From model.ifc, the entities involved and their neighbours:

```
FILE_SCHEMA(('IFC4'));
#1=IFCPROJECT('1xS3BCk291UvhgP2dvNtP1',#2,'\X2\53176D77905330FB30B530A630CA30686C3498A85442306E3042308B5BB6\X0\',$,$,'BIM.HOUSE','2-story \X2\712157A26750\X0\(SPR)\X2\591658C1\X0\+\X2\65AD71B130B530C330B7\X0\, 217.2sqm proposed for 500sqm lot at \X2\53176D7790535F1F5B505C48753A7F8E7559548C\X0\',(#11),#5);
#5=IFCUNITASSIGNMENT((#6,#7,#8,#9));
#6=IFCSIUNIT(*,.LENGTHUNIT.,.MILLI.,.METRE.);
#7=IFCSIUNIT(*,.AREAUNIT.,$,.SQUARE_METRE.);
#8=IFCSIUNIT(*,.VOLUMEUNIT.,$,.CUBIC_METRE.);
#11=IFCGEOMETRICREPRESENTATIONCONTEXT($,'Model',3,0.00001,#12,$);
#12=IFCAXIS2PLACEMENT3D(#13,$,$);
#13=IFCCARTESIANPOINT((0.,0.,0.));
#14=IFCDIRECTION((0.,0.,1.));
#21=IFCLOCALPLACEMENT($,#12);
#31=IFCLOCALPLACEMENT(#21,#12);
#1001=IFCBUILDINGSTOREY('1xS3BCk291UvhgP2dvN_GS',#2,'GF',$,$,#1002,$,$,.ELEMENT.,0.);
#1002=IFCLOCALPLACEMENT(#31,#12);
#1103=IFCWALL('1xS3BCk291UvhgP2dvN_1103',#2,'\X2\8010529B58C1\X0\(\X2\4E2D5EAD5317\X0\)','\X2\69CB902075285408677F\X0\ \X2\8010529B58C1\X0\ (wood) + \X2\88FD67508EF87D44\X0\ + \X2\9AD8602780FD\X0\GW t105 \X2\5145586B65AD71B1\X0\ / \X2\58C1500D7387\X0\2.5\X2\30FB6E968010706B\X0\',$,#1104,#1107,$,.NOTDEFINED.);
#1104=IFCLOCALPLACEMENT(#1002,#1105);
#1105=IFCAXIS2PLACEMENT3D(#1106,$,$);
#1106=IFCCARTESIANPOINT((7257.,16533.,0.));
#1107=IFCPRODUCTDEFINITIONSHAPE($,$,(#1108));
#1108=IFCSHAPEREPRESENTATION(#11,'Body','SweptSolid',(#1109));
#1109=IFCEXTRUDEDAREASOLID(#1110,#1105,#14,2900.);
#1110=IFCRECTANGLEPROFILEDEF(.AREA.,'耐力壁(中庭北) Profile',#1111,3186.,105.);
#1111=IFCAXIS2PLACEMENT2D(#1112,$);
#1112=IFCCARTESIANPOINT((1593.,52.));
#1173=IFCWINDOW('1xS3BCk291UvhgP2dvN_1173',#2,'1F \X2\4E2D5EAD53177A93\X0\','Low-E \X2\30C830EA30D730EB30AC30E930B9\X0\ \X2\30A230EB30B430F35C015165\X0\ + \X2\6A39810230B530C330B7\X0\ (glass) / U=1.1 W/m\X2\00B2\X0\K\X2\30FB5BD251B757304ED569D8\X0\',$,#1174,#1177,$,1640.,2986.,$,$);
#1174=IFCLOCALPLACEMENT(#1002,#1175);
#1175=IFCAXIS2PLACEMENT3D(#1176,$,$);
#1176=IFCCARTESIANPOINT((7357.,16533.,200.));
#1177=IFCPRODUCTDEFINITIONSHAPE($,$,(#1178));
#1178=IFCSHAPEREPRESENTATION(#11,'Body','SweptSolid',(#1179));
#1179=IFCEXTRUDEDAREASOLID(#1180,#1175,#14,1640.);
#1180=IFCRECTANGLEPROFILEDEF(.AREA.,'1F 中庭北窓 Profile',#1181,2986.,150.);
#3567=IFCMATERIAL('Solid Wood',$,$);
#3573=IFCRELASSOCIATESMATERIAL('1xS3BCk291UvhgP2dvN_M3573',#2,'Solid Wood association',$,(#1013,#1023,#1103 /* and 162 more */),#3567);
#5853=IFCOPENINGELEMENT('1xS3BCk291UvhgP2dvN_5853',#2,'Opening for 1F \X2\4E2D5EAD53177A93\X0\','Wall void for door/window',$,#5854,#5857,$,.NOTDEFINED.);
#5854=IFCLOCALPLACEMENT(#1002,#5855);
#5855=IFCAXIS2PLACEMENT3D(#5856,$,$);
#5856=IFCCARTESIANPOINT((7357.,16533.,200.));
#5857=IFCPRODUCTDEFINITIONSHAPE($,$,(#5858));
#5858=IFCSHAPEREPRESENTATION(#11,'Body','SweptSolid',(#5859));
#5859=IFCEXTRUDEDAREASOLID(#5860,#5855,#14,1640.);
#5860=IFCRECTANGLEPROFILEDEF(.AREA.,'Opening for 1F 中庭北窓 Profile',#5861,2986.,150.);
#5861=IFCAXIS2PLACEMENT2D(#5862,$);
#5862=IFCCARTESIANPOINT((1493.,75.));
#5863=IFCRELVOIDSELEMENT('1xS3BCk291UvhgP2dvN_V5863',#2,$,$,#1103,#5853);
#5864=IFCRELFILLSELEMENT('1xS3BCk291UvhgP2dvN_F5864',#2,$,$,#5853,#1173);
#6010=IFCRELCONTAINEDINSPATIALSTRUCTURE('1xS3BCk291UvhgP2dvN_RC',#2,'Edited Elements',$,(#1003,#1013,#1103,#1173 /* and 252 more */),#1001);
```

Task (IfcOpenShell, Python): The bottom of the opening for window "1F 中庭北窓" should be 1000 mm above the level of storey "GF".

```python
import numpy as np
import ifcopenshell
import ifcopenshell.api.geometry
import ifcopenshell.geom
import ifcopenshell.util.element
import ifcopenshell.util.placement
import ifcopenshell.util.shape
import ifcopenshell.util.unit

model = ifcopenshell.open("model.ifc")
unit_scale = ifcopenshell.util.unit.calculate_unit_scale(model)

window = model.by_id(1173)
opening = window.FillsVoids[0].RelatingOpeningElement
storey = ifcopenshell.util.element.get_container(window, ifc_class="IfcBuildingStorey")
level = ifcopenshell.util.placement.get_local_placement(storey.ObjectPlacement)[2, 3]

# The opening's origin need not be at the sill, so measure its lowest point.
shape = ifcopenshell.geom.create_shape(ifcopenshell.geom.settings(), opening)
bottom = ifcopenshell.util.shape.get_shape_bottom_elevation(shape, shape.geometry) / unit_scale
dz = level + 1 / unit_scale - bottom

shift = np.array([0.0, 0.0, dz])
# The window is not placed relative to its opening, so move both.
for product in (opening, window):
    matrix = ifcopenshell.util.placement.get_local_placement(product.ObjectPlacement)
    matrix[:3, 3] += shift
    ifcopenshell.api.geometry.edit_object_placement(model, product=product, matrix=matrix, is_si=False)

print(f"moved by {dz * unit_scale:+.3f} m")

model.write("model_edited.ifc")
```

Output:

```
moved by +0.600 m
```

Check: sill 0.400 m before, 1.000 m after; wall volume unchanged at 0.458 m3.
